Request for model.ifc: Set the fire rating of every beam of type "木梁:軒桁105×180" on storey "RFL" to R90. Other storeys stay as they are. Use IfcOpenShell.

First a look at what the model holds.

```python
import ifcopenshell
import ifcopenshell.util.element

model = ifcopenshell.open("model.ifc")
print(model.schema)
storey = next(s for s in model.by_type("IfcBuildingStorey") if s.Name == "RFL")
beams = [e for e in ifcopenshell.util.element.get_decomposition(storey) if e.is_a("IfcBeam")]
seen = {}
for e in beams:
    element_type = ifcopenshell.util.element.get_type(e)
    key = (element_type.Name if element_type != e and element_type else None, ifcopenshell.util.element.get_pset(e, "Pset_BeamCommon", "FireRating"))
    seen[key] = seen.get(key, 0) + 1
for (name, value), count in sorted(seen.items(), key=str):
    print(count, "x", name, "|", value)
```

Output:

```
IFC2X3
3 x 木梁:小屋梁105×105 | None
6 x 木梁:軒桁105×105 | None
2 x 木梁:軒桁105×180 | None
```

```python
import ifcopenshell
import ifcopenshell.api.pset
import ifcopenshell.util.element

model = ifcopenshell.open("model.ifc")

storey = next(s for s in model.by_type("IfcBuildingStorey") if s.Name == "RFL")
beams = [e for e in ifcopenshell.util.element.get_decomposition(storey) if e.is_a("IfcBeam")]

count = 0
for e in beams:
    element_type = ifcopenshell.util.element.get_type(e)
    if element_type in (None, e) or element_type.Name != "木梁:軒桁105×180":
        continue
    # add_pset returns the element's existing set when there is one.
    pset = ifcopenshell.api.pset.add_pset(model, product=e, name="Pset_BeamCommon")
    ifcopenshell.api.pset.edit_pset(model, pset=pset, properties={"FireRating": "R90"})
    count += 1

print(count, "beams updated")

model.write("model_edited.ifc")
```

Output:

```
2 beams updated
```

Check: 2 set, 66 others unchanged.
